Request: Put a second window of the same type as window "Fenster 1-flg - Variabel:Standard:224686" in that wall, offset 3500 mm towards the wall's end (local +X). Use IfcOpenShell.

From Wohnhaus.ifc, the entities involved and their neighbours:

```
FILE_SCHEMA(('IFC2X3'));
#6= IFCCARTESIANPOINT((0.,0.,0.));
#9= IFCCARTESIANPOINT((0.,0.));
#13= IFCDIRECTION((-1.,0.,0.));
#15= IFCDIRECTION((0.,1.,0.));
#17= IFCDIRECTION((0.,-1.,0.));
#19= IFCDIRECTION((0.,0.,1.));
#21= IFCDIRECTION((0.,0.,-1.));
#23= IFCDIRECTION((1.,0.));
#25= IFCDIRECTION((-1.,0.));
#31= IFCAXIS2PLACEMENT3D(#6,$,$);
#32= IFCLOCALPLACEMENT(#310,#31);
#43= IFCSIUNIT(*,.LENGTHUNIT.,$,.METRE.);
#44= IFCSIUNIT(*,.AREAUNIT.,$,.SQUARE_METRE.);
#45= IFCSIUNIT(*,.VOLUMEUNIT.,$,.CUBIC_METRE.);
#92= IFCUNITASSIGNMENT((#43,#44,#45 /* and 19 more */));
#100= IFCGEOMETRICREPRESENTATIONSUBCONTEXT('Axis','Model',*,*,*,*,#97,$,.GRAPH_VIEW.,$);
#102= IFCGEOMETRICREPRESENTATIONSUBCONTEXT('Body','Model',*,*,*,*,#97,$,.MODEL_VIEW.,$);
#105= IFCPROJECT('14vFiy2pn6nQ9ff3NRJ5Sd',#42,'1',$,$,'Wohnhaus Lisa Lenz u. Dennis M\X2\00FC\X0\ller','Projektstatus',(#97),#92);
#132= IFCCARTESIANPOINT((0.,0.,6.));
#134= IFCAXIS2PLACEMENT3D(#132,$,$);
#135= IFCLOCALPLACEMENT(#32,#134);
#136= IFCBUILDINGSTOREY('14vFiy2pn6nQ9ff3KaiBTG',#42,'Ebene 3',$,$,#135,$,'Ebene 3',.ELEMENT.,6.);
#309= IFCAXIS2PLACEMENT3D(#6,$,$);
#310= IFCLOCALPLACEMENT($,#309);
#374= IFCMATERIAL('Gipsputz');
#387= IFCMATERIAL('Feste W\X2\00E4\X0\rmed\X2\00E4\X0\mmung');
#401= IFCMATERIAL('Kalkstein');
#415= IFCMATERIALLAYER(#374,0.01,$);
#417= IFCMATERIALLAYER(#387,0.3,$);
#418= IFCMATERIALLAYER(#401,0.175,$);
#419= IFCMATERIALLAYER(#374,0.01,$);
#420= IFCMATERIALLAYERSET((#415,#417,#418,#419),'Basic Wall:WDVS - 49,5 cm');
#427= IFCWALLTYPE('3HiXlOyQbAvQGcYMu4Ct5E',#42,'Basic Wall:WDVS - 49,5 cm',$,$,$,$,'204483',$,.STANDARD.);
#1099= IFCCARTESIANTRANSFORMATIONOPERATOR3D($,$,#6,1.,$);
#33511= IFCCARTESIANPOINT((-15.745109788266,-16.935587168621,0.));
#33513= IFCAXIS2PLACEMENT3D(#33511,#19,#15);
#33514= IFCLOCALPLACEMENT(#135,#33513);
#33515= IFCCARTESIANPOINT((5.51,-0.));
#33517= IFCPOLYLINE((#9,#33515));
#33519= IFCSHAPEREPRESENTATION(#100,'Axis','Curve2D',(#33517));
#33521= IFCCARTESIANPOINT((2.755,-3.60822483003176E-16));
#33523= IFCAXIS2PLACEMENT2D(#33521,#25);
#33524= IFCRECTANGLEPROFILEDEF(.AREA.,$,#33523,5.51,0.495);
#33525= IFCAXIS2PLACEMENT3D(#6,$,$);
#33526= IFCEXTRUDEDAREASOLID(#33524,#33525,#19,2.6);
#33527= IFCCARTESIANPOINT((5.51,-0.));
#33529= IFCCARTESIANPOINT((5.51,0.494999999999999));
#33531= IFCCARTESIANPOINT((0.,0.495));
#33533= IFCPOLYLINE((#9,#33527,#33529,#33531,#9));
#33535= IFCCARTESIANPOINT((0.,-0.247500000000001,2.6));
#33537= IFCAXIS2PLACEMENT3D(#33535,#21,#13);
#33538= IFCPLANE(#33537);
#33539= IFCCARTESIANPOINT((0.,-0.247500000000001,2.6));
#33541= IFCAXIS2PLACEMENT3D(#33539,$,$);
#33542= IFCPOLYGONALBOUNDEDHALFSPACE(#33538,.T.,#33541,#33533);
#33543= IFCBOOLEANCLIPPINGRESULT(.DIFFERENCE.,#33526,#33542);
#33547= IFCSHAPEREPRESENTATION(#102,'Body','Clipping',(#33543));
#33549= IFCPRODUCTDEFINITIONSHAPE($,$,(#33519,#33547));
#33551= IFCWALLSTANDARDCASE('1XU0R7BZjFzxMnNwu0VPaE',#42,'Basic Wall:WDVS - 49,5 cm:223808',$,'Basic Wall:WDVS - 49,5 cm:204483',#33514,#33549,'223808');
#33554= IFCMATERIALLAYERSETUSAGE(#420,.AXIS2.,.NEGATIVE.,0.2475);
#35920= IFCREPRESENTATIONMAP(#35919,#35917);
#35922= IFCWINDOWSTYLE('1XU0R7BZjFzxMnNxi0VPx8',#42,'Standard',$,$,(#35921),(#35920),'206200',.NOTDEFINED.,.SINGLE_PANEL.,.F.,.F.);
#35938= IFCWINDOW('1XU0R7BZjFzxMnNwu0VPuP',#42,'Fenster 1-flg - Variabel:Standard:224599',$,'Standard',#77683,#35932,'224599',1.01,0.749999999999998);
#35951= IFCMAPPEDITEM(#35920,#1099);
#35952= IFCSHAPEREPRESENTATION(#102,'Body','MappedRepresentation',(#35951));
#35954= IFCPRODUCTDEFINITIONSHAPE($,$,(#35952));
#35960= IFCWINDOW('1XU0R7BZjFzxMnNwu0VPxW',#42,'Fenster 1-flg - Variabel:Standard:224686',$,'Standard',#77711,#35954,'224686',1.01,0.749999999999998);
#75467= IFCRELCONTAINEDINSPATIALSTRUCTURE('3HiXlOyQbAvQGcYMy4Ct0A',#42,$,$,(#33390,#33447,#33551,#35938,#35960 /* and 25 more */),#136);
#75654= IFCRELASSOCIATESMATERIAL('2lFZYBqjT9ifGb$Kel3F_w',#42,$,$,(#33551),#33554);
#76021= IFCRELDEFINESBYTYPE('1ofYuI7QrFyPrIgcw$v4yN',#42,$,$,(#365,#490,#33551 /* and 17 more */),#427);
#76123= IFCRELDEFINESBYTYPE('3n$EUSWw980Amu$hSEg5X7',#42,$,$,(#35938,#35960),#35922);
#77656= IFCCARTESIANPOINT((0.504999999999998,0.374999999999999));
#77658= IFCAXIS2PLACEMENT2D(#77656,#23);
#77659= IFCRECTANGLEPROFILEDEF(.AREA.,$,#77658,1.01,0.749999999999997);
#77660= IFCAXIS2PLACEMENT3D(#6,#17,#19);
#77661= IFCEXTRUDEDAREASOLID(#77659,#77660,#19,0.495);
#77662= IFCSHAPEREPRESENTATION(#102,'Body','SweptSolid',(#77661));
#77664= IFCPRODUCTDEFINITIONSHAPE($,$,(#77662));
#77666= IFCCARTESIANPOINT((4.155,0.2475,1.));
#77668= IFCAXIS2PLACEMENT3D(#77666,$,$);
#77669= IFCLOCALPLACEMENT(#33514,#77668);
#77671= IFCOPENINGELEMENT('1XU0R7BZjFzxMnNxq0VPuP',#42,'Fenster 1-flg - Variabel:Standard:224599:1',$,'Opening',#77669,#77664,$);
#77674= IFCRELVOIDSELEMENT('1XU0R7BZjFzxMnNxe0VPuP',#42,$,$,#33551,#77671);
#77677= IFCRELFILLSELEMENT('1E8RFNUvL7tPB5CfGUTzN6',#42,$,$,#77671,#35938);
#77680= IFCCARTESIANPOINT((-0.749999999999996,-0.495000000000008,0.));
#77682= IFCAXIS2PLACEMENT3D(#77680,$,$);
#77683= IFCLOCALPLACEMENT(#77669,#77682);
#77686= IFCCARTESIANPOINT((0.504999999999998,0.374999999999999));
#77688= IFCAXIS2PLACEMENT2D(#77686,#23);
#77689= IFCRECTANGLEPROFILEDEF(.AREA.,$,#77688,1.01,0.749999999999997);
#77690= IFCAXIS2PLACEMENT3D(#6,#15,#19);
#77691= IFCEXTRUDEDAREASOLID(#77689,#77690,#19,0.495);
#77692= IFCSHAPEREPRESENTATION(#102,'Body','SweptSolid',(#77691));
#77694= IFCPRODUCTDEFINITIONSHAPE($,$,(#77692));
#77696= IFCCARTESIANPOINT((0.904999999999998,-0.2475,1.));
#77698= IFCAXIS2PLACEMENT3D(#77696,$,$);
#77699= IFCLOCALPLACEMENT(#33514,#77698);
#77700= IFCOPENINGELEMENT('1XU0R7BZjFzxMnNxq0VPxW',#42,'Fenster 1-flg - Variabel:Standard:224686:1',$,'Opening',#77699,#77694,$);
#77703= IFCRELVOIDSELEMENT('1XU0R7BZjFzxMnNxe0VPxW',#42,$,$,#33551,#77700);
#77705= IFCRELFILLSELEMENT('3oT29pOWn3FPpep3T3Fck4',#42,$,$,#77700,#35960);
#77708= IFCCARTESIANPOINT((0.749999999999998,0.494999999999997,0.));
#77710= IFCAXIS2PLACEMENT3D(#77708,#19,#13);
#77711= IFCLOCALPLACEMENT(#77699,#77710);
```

```python
import ifcopenshell
import ifcopenshell.api.feature
import ifcopenshell.api.geometry
import ifcopenshell.api.root
import ifcopenshell.geom
import ifcopenshell.util.element
import ifcopenshell.util.placement
import ifcopenshell.util.shape

model = ifcopenshell.open("Wohnhaus.ifc")
settings = ifcopenshell.geom.settings()


def volume(element):
    """Net volume in cubic metres, openings subtracted."""
    shape = ifcopenshell.geom.create_shape(settings, element)
    return ifcopenshell.util.shape.get_volume(shape.geometry)


def reuse_history(source, copy):
    """copy_class also copies each property set's owner history, people and application; keep the originals."""
    for rel in copy.IsDefinedBy:
        if rel.is_a("IfcRelDefinesByProperties") and (history := rel.RelatingPropertyDefinition.OwnerHistory):
            rel.RelatingPropertyDefinition.OwnerHistory = source.OwnerHistory
            ifcopenshell.util.element.remove_deep2(model, history)


window = model.by_guid("1XU0R7BZjFzxMnNwu0VPxW")
opening = window.FillsVoids[0].RelatingOpeningElement
wall = opening.VoidsElements[0].RelatingBuildingElement
before = volume(wall)
shift = ifcopenshell.util.placement.get_local_placement(wall.ObjectPlacement)[:3, 0] * 3.5

# copy_class copies the void relationship, type, container and properties, but no geometry.
new_opening = ifcopenshell.api.root.copy_class(model, product=opening)
new_opening.Representation = ifcopenshell.util.element.copy_deep(
    model, opening.Representation, exclude=["IfcGeometricRepresentationContext", "IfcRepresentationMap"]
)
new_opening.Name = "Fenster 1-flg - Variabel:Standard"
new_window = ifcopenshell.api.root.copy_class(model, product=window)
new_window.Representation = ifcopenshell.util.element.copy_deep(
    model, window.Representation, exclude=["IfcGeometricRepresentationContext", "IfcRepresentationMap"]
)
new_window.Name = "Fenster 1-flg - Variabel:Standard"
new_window.Tag = None
reuse_history(window, new_window)
fills = ifcopenshell.api.feature.add_filling(model, opening=new_opening, element=new_window)
fills.OwnerHistory = new_window.OwnerHistory  # required in IFC2X3

for old, new in ((opening, new_opening), (window, new_window)):
    matrix = ifcopenshell.util.placement.get_local_placement(old.ObjectPlacement)
    matrix[:3, 3] += shift
    ifcopenshell.api.geometry.edit_object_placement(model, product=new, matrix=matrix, is_si=False)

after = volume(wall)

print(f"wall volume {before:.3f} -> {after:.3f} m3")

model.write("Wohnhaus_edited.ifc")
```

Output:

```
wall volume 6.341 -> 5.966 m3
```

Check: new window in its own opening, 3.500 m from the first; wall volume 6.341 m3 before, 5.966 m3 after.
